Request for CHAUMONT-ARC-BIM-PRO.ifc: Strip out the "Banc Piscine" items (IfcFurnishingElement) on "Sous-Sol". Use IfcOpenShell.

First a look at what the model holds.

```python
import ifcopenshell
import ifcopenshell.util.element

model = ifcopenshell.open("CHAUMONT-ARC-BIM-PRO.ifc")
print(model.schema)
storey = next(s for s in model.by_type("IfcBuildingStorey") if s.Name == "Sous-Sol")
furniture = [e for e in ifcopenshell.util.element.get_decomposition(storey) if e.is_a("IfcFurnishingElement")]
seen = {}
for e in furniture:
    element_type = ifcopenshell.util.element.get_type(e)
    name = element_type.Name if element_type not in (None, e) else None
    seen[name] = seen.get(name, 0) + 1
for name, count in sorted(seen.items(), key=str):
    print(count, "x", name)
```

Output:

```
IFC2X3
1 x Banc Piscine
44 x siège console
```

```python
import ifcopenshell
import ifcopenshell.api.root
import ifcopenshell.util.element

model = ifcopenshell.open("CHAUMONT-ARC-BIM-PRO.ifc")

storey = next(s for s in model.by_type("IfcBuildingStorey") if s.Name == "Sous-Sol")
furniture = [e for e in ifcopenshell.util.element.get_decomposition(storey) if e.is_a("IfcFurnishingElement")]
targets = [e for e in furniture if (t := ifcopenshell.util.element.get_type(e)) not in (None, e) and t.Name == "Banc Piscine"]

for e in targets:
    ifcopenshell.api.root.remove_product(model, product=e)
print(len(targets), "removed")

model.write("CHAUMONT-ARC-BIM-PRO_v2.ifc")
```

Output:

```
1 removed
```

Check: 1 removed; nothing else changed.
